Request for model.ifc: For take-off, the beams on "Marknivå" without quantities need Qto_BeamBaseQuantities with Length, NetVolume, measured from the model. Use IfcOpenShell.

First a look at what the model holds.

```python
import ifcopenshell
import ifcopenshell.util.element
import ifcopenshell.util.unit

model = ifcopenshell.open("model.ifc")
print(model.schema)
for unit_type in ("LENGTHUNIT", "AREAUNIT", "VOLUMEUNIT"):
    print(unit_type, ifcopenshell.util.unit.calculate_unit_scale(model, unit_type))
storey = next(s for s in model.by_type("IfcBuildingStorey") if s.Name == "Marknivå")
beams = [e for e in ifcopenshell.util.element.get_decomposition(storey) if e.is_a("IfcBeam")]
for e in sorted(beams, key=lambda e: e.id()):
    print(e.id(), e.is_a(), e.Name, list(ifcopenshell.util.element.get_psets(e, qtos_only=True)), sep=" | ")
```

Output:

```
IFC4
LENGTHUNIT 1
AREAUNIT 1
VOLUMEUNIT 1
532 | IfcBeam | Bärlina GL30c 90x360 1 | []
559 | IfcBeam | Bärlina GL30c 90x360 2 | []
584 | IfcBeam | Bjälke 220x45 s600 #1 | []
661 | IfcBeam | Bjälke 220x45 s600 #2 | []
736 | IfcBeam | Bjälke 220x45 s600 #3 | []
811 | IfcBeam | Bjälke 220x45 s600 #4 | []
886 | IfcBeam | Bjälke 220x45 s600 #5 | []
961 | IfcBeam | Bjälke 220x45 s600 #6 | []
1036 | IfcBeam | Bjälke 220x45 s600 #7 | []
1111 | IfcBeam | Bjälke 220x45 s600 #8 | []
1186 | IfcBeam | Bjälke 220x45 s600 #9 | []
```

```python
import ifcopenshell
import ifcopenshell.api.pset
import ifcopenshell.geom
import ifcopenshell.util.element
import ifcopenshell.util.shape
import ifcopenshell.util.unit

model = ifcopenshell.open("model.ifc")
unit_scale = ifcopenshell.util.unit.calculate_unit_scale(model)
volume_scale = ifcopenshell.util.unit.calculate_unit_scale(model, "VOLUMEUNIT")
settings = ifcopenshell.geom.settings()

storey = next(s for s in model.by_type("IfcBuildingStorey") if s.Name == "Marknivå")
beams = [e for e in ifcopenshell.util.element.get_decomposition(storey) if e.is_a("IfcBeam")]

for e in sorted(beams, key=lambda e: e.id()):
    if ifcopenshell.util.element.get_psets(e, qtos_only=True, should_inherit=False):
        continue
    # Geometry comes back in metres, in the element's own axes.
    shape = ifcopenshell.geom.create_shape(settings, e)
    values = {
        "Length": ifcopenshell.util.shape.get_max_xyz(shape.geometry) / unit_scale,
        "NetVolume": ifcopenshell.util.shape.get_volume(shape.geometry) / volume_scale,
    }
    qto = ifcopenshell.api.pset.add_qto(model, product=e, name="Qto_BeamBaseQuantities")
    ifcopenshell.api.pset.edit_qto(model, qto=qto, properties=values)
    print(e.id(), {k: round(v, 3) for k, v in values.items()})

model.write("model_edited.ifc")
```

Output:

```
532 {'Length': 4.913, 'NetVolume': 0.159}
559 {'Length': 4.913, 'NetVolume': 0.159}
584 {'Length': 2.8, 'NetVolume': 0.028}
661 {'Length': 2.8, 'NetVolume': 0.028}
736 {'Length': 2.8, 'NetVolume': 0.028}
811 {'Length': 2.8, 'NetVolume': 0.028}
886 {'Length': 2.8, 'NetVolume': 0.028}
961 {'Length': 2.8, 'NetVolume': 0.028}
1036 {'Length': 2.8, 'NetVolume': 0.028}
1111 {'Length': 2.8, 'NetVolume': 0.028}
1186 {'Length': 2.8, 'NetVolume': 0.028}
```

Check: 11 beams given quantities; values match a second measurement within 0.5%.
